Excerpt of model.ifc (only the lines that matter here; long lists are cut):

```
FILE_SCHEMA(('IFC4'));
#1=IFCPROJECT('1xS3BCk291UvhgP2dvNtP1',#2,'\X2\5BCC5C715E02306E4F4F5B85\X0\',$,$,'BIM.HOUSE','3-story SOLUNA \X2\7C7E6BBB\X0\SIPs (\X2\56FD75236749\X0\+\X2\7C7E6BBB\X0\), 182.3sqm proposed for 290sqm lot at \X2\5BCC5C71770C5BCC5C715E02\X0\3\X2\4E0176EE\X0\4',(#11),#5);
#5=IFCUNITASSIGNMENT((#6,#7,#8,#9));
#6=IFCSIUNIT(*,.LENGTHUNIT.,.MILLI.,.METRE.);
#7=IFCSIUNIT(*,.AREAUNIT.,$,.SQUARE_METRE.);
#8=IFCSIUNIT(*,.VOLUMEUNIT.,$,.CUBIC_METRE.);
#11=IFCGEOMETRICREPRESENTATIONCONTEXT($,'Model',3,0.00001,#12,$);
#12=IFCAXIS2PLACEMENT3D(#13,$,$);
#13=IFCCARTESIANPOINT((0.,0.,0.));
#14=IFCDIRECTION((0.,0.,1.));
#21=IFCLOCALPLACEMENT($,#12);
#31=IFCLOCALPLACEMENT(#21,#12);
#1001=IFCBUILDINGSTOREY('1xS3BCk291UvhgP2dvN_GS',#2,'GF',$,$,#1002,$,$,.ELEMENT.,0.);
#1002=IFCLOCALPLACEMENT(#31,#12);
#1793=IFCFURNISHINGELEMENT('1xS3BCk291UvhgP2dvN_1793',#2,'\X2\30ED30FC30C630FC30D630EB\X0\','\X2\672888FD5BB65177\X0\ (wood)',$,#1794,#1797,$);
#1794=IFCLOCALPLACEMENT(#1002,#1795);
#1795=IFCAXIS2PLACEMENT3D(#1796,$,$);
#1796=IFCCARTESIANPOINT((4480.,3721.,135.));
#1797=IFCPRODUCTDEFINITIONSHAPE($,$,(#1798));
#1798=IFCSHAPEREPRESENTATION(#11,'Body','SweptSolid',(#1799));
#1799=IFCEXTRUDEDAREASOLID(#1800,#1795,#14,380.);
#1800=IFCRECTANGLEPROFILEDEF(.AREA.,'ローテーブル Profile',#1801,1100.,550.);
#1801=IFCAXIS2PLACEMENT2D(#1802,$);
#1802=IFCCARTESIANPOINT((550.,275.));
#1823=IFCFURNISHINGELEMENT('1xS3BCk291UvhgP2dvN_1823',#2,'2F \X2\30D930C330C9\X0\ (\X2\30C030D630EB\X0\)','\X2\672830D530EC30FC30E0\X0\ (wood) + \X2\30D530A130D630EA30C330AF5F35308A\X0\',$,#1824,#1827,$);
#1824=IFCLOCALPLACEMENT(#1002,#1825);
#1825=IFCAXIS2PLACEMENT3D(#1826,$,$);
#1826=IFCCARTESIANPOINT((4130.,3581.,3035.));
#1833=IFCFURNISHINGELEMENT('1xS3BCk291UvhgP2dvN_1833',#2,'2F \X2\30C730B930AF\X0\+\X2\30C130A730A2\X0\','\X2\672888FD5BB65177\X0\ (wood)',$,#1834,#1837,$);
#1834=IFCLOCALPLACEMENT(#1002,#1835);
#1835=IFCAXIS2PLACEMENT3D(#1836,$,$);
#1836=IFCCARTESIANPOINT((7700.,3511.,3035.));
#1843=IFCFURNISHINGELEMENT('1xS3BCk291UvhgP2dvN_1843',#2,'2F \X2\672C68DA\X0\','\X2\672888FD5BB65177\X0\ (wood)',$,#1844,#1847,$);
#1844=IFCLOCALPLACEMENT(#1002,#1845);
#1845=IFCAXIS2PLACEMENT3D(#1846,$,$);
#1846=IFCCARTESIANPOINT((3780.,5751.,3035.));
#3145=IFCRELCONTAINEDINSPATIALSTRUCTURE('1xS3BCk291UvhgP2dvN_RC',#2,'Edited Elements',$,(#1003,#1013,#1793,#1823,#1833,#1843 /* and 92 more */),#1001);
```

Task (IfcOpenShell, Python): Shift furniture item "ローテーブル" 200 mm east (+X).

```python
import ifcopenshell
import ifcopenshell.api.geometry
import ifcopenshell.util.placement
import ifcopenshell.util.unit

model = ifcopenshell.open("model.ifc")
unit_scale = ifcopenshell.util.unit.calculate_unit_scale(model)

item = model.by_guid("1xS3BCk291UvhgP2dvN_1793")
matrix = ifcopenshell.util.placement.get_local_placement(item.ObjectPlacement)
matrix[0, 3] += 0.2 / unit_scale
ifcopenshell.api.geometry.edit_object_placement(model, product=item, matrix=matrix, is_si=False)

print(ifcopenshell.util.placement.get_local_placement(item.ObjectPlacement).round(3) + 0.0)

model.write("model-out.ifc")
```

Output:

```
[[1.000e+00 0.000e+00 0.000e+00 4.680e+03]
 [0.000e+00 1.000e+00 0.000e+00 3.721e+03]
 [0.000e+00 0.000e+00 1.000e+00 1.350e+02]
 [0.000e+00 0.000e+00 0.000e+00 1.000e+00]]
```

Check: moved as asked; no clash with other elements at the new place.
